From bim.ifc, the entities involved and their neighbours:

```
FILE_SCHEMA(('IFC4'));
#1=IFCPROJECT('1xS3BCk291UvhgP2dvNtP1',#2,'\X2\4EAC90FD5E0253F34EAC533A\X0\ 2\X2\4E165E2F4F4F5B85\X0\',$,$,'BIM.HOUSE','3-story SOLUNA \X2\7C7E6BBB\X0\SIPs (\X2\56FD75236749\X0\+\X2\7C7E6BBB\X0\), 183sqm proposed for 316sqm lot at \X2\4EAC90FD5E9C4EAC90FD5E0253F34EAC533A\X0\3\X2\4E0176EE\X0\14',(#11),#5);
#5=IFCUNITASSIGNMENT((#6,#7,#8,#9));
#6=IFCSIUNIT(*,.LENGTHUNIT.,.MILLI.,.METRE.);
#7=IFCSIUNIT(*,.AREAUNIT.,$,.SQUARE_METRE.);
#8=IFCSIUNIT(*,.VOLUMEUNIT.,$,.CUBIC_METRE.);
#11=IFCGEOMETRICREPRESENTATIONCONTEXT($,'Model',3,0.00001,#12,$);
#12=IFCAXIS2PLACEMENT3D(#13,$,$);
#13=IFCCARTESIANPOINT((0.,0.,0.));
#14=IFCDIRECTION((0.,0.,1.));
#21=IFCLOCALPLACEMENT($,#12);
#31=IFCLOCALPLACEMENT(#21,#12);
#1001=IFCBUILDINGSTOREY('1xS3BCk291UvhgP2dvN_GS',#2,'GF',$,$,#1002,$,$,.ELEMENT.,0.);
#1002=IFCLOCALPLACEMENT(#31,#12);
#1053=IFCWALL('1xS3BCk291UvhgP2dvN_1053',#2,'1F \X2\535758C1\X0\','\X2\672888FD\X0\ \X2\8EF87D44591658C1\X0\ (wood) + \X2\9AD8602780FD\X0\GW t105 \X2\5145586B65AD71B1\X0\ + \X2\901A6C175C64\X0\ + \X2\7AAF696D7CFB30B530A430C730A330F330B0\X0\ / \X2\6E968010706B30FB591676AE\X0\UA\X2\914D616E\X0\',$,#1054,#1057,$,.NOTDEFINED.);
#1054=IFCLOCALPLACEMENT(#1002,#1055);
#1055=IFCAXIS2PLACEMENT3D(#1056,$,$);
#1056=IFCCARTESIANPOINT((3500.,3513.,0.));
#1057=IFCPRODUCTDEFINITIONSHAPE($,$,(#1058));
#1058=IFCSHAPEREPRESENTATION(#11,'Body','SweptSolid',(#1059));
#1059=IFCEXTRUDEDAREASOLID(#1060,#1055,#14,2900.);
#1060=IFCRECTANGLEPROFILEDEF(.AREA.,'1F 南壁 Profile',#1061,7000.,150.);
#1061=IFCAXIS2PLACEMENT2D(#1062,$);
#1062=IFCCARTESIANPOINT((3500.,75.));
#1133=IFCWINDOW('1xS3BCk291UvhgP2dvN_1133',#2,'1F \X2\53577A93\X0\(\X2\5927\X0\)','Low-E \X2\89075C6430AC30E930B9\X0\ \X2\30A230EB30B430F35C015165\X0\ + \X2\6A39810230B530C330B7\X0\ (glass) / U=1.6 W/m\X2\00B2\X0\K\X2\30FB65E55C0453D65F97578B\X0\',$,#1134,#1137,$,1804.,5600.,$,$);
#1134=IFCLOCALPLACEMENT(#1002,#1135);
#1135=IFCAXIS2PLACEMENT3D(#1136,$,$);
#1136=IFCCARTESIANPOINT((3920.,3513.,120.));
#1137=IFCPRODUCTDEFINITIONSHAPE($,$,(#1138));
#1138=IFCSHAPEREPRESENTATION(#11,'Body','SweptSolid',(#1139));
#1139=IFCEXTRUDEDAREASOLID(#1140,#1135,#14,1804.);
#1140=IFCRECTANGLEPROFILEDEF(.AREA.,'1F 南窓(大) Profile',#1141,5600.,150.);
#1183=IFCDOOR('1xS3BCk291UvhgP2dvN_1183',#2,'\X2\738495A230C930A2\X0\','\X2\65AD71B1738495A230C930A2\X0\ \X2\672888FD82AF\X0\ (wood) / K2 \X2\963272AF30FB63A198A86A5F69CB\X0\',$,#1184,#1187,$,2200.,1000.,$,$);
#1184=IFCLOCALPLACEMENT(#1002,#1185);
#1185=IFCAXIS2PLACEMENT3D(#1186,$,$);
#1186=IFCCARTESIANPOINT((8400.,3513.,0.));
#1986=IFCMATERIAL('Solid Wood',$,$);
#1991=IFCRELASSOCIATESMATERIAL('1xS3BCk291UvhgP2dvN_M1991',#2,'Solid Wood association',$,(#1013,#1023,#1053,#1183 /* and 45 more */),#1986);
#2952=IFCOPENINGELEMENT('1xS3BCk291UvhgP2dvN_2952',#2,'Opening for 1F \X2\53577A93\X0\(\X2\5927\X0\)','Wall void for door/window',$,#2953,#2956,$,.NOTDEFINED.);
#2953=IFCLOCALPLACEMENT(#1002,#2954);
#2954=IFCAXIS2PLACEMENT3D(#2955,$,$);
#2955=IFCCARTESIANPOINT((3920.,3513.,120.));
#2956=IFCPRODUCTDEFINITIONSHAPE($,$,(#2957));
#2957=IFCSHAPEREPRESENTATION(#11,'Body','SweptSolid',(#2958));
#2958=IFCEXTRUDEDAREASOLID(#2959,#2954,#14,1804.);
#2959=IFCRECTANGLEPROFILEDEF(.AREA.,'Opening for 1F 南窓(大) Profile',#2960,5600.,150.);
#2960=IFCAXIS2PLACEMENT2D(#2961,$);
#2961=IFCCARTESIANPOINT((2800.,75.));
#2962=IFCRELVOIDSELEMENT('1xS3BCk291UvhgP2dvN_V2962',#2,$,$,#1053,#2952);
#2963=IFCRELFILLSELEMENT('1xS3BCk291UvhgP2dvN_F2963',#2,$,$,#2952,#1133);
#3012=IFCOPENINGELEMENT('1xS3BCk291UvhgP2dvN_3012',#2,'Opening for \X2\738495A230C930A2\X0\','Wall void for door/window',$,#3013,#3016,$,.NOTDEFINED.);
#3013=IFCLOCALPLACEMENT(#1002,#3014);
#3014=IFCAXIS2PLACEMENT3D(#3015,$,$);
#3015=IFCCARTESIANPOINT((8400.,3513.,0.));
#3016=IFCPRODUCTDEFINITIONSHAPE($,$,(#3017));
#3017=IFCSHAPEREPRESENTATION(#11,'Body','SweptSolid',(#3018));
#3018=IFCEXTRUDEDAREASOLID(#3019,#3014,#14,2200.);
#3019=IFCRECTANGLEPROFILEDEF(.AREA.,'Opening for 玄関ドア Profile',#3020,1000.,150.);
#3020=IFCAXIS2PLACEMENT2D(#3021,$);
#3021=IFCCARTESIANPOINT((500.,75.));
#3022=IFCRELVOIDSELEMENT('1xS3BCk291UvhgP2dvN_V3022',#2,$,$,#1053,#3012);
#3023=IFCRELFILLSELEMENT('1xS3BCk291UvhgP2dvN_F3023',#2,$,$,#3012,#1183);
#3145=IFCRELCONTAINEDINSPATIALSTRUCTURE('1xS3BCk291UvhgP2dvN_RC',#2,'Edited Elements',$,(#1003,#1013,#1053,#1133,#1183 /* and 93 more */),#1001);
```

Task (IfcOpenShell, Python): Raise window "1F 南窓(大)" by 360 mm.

```python
import numpy as np
import ifcopenshell
import ifcopenshell.api.geometry
import ifcopenshell.util.placement
import ifcopenshell.util.unit

model = ifcopenshell.open("bim.ifc")
unit_scale = ifcopenshell.util.unit.calculate_unit_scale(model)

window = model.by_guid("1xS3BCk291UvhgP2dvN_1133")
opening = window.FillsVoids[0].RelatingOpeningElement
dz = 0.36 / unit_scale

shift = np.array([0.0, 0.0, dz])
# The window is not placed relative to its opening, so move both.
for product in (opening, window):
    matrix = ifcopenshell.util.placement.get_local_placement(product.ObjectPlacement)
    matrix[:3, 3] += shift
    ifcopenshell.api.geometry.edit_object_placement(model, product=product, matrix=matrix, is_si=False)

print(f"moved by {dz * unit_scale:+.3f} m")

model.write("bim_edited.ifc")
```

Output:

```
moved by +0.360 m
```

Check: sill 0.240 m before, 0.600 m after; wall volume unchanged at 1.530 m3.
